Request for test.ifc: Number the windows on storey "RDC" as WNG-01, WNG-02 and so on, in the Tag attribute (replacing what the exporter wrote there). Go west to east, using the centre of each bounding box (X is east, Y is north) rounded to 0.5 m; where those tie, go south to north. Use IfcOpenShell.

First a look at what the model holds.

```python
import ifcopenshell
import ifcopenshell.util.element
import ifcopenshell.util.placement

model = ifcopenshell.open("test.ifc")
print(model.schema)
storey = next(s for s in model.by_type("IfcBuildingStorey") if s.Name == "RDC")
windows = [e for e in ifcopenshell.util.element.get_decomposition(storey) if e.is_a("IfcWindow")]
for e in sorted(windows, key=lambda e: e.id()):
    origin = ifcopenshell.util.placement.get_local_placement(e.ObjectPlacement)[:3, 3]
    print(e.id(), e.Tag, e.Name, origin.round(2) + 0.0, sep=" | ")
```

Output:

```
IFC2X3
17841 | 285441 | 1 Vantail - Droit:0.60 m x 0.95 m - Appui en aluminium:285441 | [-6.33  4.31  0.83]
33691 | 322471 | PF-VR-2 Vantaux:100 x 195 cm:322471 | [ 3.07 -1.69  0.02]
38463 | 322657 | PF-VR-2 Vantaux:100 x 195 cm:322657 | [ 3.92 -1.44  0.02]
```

```python
import ifcopenshell
import ifcopenshell.geom
import ifcopenshell.util.element
import ifcopenshell.util.shape

model = ifcopenshell.open("test.ifc")
settings = ifcopenshell.geom.settings()
settings.set("use-world-coords", True)


def centre(element):
    shape = ifcopenshell.geom.create_shape(settings, element)
    return ifcopenshell.util.shape.get_bbox_centroid(shape.geometry)


storey = next(s for s in model.by_type("IfcBuildingStorey") if s.Name == "RDC")
windows = [e for e in ifcopenshell.util.element.get_decomposition(storey) if e.is_a("IfcWindow")]

# Insertion points can sit at a corner or the storey origin, so sort by the geometry (in metres).
centres = {e: centre(e) for e in windows}
windows.sort(key=lambda e: (round(centres[e][0] / 0.5), centres[e][1]))

for i, e in enumerate(windows, start=1):
    number = f"WNG-{i:02d}"
    e.Tag = number
    print(e.id(), number)

model.write("test_edited.ifc")
```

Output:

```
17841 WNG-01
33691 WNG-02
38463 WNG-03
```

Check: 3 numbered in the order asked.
